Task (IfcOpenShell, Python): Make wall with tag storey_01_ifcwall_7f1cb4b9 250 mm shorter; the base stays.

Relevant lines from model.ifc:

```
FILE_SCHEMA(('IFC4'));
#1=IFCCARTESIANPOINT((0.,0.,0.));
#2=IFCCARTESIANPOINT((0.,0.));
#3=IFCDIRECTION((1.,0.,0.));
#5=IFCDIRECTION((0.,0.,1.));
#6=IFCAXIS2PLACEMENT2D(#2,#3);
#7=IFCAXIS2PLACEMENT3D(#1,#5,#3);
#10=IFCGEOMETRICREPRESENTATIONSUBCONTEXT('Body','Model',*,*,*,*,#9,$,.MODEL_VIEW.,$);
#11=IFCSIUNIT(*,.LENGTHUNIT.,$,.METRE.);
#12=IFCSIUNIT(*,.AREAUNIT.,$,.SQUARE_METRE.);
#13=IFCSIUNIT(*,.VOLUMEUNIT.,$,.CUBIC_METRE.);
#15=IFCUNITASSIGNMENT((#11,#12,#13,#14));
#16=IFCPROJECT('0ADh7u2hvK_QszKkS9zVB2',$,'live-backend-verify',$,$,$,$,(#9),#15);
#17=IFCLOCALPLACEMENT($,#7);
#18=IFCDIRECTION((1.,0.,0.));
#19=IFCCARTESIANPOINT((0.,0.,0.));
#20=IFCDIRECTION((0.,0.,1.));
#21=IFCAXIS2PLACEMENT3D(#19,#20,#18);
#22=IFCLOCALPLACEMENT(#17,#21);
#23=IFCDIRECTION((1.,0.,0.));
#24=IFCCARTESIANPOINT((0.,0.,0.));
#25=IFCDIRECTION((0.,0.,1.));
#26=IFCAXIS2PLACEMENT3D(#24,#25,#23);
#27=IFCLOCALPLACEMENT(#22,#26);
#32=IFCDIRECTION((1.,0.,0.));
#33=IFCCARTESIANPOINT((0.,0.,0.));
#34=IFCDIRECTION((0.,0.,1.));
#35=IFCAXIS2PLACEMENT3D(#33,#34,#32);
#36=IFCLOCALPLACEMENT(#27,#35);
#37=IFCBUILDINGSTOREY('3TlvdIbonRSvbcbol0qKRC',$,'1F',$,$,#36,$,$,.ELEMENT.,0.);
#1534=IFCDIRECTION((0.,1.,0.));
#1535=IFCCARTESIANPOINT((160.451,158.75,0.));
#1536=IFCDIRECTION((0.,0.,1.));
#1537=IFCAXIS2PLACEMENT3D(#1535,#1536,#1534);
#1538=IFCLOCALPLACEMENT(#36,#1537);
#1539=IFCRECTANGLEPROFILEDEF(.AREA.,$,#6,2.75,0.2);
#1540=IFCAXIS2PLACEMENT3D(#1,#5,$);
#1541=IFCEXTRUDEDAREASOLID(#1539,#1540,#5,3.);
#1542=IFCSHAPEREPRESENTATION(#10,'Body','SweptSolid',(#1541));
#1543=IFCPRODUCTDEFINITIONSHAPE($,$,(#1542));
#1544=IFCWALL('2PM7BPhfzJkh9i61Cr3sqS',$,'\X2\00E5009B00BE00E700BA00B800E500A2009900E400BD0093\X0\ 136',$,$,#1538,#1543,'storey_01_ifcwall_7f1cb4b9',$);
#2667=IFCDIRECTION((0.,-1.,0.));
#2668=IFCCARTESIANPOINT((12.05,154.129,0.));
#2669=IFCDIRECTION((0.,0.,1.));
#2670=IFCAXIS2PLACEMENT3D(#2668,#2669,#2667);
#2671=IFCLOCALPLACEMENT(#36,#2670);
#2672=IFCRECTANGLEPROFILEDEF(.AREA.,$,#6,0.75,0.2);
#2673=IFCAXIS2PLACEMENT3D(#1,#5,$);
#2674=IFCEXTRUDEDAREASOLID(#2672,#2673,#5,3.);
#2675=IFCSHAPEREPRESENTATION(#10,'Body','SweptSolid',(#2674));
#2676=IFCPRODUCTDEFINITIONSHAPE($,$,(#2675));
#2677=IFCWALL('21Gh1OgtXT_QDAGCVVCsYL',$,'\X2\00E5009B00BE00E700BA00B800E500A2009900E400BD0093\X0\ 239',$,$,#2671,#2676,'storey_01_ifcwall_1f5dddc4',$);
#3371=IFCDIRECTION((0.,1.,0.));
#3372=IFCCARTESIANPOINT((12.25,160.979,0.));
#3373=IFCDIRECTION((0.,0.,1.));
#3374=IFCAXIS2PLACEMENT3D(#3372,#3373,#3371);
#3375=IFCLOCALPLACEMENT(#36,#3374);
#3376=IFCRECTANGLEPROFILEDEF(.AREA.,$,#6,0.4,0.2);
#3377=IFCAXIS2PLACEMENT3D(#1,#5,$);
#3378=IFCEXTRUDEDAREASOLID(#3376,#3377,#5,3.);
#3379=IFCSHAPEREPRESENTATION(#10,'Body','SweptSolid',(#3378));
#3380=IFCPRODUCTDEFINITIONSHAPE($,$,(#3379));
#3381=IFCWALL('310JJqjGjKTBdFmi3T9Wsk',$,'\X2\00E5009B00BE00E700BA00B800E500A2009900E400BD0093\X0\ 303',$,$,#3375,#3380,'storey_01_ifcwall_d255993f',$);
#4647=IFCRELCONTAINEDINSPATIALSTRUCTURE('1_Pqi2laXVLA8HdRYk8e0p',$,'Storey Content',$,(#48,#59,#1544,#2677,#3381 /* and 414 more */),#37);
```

```python
import ifcopenshell
import ifcopenshell.geom
import ifcopenshell.util.representation
import ifcopenshell.util.shape
import ifcopenshell.util.unit

model = ifcopenshell.open("model.ifc")
unit_scale = ifcopenshell.util.unit.calculate_unit_scale(model)
settings = ifcopenshell.geom.settings()


def volume(element):
    """Net volume in cubic metres, openings subtracted."""
    shape = ifcopenshell.geom.create_shape(settings, element)
    return ifcopenshell.util.shape.get_volume(shape.geometry)


wall = model.by_guid("2PM7BPhfzJkh9i61Cr3sqS")
before = volume(wall)

body = ifcopenshell.util.representation.get_representation(wall, "Model", "Body")
solid = body.Items[0]
old_height = solid.Depth
solid.Depth -= 0.25 / unit_scale
after = volume(wall)

print(f"height {old_height:g} -> {solid.Depth:g}, volume {before:.3f} -> {after:.3f} m3")

model.write("model-out.ifc")
```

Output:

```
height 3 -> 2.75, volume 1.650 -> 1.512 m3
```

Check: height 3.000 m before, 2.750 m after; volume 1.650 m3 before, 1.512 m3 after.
